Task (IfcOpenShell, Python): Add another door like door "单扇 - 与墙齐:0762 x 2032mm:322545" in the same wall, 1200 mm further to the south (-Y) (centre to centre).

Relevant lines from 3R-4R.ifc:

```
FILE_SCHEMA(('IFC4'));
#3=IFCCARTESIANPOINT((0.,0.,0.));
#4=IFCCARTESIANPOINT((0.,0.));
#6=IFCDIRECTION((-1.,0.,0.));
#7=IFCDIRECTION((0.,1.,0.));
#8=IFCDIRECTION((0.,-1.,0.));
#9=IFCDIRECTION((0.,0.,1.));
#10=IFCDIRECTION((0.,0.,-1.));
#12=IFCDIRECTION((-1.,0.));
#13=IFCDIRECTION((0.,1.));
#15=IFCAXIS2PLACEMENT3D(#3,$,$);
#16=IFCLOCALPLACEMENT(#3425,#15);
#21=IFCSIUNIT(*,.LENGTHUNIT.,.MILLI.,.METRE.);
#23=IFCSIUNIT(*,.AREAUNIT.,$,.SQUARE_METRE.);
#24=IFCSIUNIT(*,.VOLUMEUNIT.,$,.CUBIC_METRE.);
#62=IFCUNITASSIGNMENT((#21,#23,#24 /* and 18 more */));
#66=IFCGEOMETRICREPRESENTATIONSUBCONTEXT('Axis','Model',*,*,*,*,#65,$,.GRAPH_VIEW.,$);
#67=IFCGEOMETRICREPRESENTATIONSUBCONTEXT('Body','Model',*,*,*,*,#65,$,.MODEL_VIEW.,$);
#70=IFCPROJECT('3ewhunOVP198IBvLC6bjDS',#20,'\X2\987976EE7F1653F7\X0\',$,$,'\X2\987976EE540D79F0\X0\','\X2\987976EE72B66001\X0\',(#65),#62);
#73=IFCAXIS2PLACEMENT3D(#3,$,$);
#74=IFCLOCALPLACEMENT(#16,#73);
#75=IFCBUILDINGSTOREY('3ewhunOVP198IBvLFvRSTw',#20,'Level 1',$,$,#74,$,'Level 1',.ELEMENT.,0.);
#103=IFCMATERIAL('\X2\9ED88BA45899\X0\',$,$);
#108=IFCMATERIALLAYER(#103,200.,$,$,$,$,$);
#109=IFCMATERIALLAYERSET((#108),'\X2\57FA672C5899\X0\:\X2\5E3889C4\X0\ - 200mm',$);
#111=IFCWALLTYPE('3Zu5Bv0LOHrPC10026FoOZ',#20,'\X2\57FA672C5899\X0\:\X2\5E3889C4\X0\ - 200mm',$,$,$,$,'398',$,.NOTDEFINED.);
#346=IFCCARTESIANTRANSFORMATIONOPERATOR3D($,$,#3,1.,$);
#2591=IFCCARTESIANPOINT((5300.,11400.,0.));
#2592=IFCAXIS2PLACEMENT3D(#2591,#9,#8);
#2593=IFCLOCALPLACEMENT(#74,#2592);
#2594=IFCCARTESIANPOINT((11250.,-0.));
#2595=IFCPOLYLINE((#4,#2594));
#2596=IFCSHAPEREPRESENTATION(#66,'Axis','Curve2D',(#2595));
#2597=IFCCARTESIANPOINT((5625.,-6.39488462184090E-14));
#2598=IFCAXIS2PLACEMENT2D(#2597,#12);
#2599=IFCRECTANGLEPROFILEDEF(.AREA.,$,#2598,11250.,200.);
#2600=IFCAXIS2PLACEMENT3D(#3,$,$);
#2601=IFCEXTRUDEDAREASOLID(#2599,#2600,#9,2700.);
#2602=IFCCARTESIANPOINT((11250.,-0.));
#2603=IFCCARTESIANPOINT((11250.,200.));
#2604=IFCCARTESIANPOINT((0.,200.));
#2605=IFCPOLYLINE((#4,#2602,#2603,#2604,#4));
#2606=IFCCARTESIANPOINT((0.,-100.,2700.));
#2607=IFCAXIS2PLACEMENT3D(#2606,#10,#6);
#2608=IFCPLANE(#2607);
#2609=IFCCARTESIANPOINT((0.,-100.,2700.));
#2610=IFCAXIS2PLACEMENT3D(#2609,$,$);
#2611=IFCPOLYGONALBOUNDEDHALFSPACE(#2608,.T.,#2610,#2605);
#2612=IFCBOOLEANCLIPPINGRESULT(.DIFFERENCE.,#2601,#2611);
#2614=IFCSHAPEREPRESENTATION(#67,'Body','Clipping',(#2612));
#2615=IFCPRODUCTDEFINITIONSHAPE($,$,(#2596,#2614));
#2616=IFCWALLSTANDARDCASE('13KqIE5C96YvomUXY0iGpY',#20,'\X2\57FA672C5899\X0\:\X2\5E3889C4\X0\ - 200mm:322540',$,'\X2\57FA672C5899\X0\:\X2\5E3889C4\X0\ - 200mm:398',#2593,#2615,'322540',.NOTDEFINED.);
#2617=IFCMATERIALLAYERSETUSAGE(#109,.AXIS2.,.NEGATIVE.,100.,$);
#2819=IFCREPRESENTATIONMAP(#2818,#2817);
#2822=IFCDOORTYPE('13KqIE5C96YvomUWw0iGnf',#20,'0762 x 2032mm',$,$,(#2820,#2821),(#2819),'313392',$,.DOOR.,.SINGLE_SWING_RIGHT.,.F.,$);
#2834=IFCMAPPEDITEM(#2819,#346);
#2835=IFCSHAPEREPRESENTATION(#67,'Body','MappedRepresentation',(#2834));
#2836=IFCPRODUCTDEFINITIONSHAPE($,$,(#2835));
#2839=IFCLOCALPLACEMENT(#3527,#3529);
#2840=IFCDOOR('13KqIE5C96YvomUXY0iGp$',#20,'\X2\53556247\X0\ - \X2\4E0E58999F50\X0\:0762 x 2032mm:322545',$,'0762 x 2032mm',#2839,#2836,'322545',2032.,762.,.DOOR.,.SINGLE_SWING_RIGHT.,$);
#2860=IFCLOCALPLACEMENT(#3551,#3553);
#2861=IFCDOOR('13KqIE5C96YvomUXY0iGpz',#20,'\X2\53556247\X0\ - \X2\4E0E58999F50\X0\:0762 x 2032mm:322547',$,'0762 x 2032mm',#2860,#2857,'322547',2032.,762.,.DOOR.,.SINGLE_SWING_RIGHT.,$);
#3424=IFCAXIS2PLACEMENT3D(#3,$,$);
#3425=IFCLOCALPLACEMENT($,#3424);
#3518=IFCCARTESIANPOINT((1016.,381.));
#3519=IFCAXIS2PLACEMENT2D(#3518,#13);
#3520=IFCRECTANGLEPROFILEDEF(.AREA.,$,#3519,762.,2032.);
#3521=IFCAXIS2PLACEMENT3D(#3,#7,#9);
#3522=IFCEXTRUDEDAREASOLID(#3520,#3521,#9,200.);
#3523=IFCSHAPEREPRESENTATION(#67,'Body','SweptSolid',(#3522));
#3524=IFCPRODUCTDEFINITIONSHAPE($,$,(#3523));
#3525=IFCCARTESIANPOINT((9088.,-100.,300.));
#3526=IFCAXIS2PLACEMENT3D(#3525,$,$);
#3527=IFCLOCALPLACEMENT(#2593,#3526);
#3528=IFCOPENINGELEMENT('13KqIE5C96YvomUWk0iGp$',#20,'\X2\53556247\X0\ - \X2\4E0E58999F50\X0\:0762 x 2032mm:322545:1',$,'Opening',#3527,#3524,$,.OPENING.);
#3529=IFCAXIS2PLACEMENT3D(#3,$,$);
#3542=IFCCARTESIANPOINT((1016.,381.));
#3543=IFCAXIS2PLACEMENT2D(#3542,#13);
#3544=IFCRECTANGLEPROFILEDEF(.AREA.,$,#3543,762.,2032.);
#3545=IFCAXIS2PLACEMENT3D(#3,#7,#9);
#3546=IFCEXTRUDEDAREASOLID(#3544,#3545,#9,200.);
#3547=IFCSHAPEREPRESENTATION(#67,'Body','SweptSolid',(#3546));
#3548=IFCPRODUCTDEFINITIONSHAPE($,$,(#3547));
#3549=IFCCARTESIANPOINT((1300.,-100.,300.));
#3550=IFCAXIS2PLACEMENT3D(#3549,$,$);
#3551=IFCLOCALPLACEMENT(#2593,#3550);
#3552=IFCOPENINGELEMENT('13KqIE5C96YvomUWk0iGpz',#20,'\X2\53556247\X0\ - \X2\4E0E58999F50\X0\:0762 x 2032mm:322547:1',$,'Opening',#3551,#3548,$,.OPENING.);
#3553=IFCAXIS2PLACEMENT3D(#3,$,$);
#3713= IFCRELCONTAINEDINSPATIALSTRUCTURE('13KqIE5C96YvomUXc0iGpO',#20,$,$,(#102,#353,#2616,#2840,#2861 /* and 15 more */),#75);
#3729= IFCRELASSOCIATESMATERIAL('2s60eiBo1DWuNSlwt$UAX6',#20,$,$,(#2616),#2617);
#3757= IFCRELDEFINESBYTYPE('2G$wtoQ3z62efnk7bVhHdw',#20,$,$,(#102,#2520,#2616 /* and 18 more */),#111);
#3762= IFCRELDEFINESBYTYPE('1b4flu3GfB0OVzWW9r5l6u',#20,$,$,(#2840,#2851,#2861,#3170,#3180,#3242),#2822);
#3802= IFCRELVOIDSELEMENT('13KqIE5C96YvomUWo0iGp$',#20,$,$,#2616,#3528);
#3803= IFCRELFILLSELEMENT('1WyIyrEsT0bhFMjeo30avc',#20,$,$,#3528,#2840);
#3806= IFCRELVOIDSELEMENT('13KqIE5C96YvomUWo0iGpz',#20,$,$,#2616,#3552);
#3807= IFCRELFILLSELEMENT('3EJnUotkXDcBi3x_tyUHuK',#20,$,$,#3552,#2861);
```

```python
import ifcopenshell
import ifcopenshell.api.feature
import ifcopenshell.api.geometry
import ifcopenshell.api.root
import ifcopenshell.geom
import ifcopenshell.util.element
import ifcopenshell.util.placement
import ifcopenshell.util.shape
import ifcopenshell.util.unit

model = ifcopenshell.open("3R-4R.ifc")
unit_scale = ifcopenshell.util.unit.calculate_unit_scale(model)
settings = ifcopenshell.geom.settings()


def volume(element):
    """Net volume in cubic metres, openings subtracted."""
    shape = ifcopenshell.geom.create_shape(settings, element)
    return ifcopenshell.util.shape.get_volume(shape.geometry)


def reuse_history(source, copy):
    """copy_class also copies each property set's owner history, people and application; keep the originals."""
    for rel in copy.IsDefinedBy:
        if rel.is_a("IfcRelDefinesByProperties") and (history := rel.RelatingPropertyDefinition.OwnerHistory):
            rel.RelatingPropertyDefinition.OwnerHistory = source.OwnerHistory
            ifcopenshell.util.element.remove_deep2(model, history)


door = model.by_guid("13KqIE5C96YvomUXY0iGp$")
opening = door.FillsVoids[0].RelatingOpeningElement
wall = opening.VoidsElements[0].RelatingBuildingElement
before = volume(wall)
shift = ifcopenshell.util.placement.get_local_placement(wall.ObjectPlacement)[:3, 0] * 1.2 / unit_scale

# copy_class copies the void relationship, type, container and properties, but no geometry.
new_opening = ifcopenshell.api.root.copy_class(model, product=opening)
new_opening.Representation = ifcopenshell.util.element.copy_deep(
    model, opening.Representation, exclude=["IfcGeometricRepresentationContext", "IfcRepresentationMap"]
)
new_opening.Name = "单扇 - 与墙齐:0762 x 2032mm"
new_door = ifcopenshell.api.root.copy_class(model, product=door)
new_door.Representation = ifcopenshell.util.element.copy_deep(
    model, door.Representation, exclude=["IfcGeometricRepresentationContext", "IfcRepresentationMap"]
)
new_door.Name = "单扇 - 与墙齐:0762 x 2032mm"
new_door.Tag = None
reuse_history(door, new_door)
ifcopenshell.api.feature.add_filling(model, opening=new_opening, element=new_door)

for old, new in ((opening, new_opening), (door, new_door)):
    matrix = ifcopenshell.util.placement.get_local_placement(old.ObjectPlacement)
    matrix[:3, 3] += shift
    ifcopenshell.api.geometry.edit_object_placement(model, product=new, matrix=matrix, is_si=False)

after = volume(wall)

print(f"wall volume {before:.3f} -> {after:.3f} m3")

model.write("3R-4R_updated.ifc")
```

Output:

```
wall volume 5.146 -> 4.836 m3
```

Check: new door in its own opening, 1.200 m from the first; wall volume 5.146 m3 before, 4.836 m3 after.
